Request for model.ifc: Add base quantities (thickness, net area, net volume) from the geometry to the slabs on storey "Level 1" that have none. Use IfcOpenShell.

First a look at what the model holds.

```python
import ifcopenshell
import ifcopenshell.util.element
import ifcopenshell.util.unit

model = ifcopenshell.open("model.ifc")
print(model.schema)
for unit_type in ("LENGTHUNIT", "AREAUNIT", "VOLUMEUNIT"):
    print(unit_type, ifcopenshell.util.unit.calculate_unit_scale(model, unit_type))
storey = next(s for s in model.by_type("IfcBuildingStorey") if s.Name == "Level 1")
slabs = [e for e in ifcopenshell.util.element.get_decomposition(storey) if e.is_a("IfcSlab")]
for e in sorted(slabs, key=lambda e: e.id()):
    print(e.id(), e.is_a(), e.Name, list(ifcopenshell.util.element.get_psets(e, qtos_only=True)), sep=" | ")
```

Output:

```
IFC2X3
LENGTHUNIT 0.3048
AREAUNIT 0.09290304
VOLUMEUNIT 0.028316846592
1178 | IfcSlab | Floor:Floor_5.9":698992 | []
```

```python
import ifcopenshell
import ifcopenshell.api.pset
import ifcopenshell.geom
import ifcopenshell.util.element
import ifcopenshell.util.shape
import ifcopenshell.util.unit

model = ifcopenshell.open("model.ifc")
unit_scale = ifcopenshell.util.unit.calculate_unit_scale(model)
area_scale = ifcopenshell.util.unit.calculate_unit_scale(model, "AREAUNIT")
volume_scale = ifcopenshell.util.unit.calculate_unit_scale(model, "VOLUMEUNIT")
settings = ifcopenshell.geom.settings()

storey = next(s for s in model.by_type("IfcBuildingStorey") if s.Name == "Level 1")
slabs = [e for e in ifcopenshell.util.element.get_decomposition(storey) if e.is_a("IfcSlab")]

for e in sorted(slabs, key=lambda e: e.id()):
    if ifcopenshell.util.element.get_psets(e, qtos_only=True, should_inherit=False):
        continue
    # Geometry comes back in metres, in the element's own axes.
    shape = ifcopenshell.geom.create_shape(settings, e)
    values = {
        "Width": ifcopenshell.util.shape.get_z(shape.geometry) / unit_scale,
        "NetArea": ifcopenshell.util.shape.get_footprint_area(shape.geometry) / area_scale,
        "NetVolume": ifcopenshell.util.shape.get_volume(shape.geometry) / volume_scale,
    }
    qto = ifcopenshell.api.pset.add_qto(model, product=e, name="BaseQuantities")
    ifcopenshell.api.pset.edit_qto(model, qto=qto, properties=values)
    print(e.id(), {k: round(v, 3) for k, v in values.items()})

model.write("model_edited.ifc")
```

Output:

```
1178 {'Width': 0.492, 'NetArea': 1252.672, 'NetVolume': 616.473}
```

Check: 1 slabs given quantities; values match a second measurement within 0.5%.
